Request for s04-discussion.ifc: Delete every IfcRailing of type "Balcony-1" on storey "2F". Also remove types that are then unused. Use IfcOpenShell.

First a look at what the model holds.

```python
import ifcopenshell
import ifcopenshell.util.element

model = ifcopenshell.open("s04-discussion.ifc")
print(model.schema)
storey = next(s for s in model.by_type("IfcBuildingStorey") if s.Name == "2F")
railings = [e for e in ifcopenshell.util.element.get_decomposition(storey) if e.is_a("IfcRailing")]
seen = {}
for e in railings:
    element_type = ifcopenshell.util.element.get_type(e)
    name = element_type.Name if element_type not in (None, e) else None
    seen[name] = seen.get(name, 0) + 1
for name, count in sorted(seen.items(), key=str):
    print(count, "x", name)
```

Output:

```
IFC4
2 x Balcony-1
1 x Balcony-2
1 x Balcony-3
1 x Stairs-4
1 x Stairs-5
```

```python
import ifcopenshell
import ifcopenshell.api.root
import ifcopenshell.util.element

model = ifcopenshell.open("s04-discussion.ifc")

storey = next(s for s in model.by_type("IfcBuildingStorey") if s.Name == "2F")
railings = [e for e in ifcopenshell.util.element.get_decomposition(storey) if e.is_a("IfcRailing")]
targets = [e for e in railings if (t := ifcopenshell.util.element.get_type(e)) not in (None, e) and t.Name == "Balcony-1"]
types = {ifcopenshell.util.element.get_type(e) for e in targets} - {None, *targets}

for e in targets:
    ifcopenshell.api.root.remove_product(model, product=e)
print(len(targets), "removed")

unused = [t for t in types if not ifcopenshell.util.element.get_types(t)]
for t in unused:
    ifcopenshell.api.root.remove_product(model, product=t)
print(len(unused), "unused types removed")

model.write("s04-discussion-out.ifc")
```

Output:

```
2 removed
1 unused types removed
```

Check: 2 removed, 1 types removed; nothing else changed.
